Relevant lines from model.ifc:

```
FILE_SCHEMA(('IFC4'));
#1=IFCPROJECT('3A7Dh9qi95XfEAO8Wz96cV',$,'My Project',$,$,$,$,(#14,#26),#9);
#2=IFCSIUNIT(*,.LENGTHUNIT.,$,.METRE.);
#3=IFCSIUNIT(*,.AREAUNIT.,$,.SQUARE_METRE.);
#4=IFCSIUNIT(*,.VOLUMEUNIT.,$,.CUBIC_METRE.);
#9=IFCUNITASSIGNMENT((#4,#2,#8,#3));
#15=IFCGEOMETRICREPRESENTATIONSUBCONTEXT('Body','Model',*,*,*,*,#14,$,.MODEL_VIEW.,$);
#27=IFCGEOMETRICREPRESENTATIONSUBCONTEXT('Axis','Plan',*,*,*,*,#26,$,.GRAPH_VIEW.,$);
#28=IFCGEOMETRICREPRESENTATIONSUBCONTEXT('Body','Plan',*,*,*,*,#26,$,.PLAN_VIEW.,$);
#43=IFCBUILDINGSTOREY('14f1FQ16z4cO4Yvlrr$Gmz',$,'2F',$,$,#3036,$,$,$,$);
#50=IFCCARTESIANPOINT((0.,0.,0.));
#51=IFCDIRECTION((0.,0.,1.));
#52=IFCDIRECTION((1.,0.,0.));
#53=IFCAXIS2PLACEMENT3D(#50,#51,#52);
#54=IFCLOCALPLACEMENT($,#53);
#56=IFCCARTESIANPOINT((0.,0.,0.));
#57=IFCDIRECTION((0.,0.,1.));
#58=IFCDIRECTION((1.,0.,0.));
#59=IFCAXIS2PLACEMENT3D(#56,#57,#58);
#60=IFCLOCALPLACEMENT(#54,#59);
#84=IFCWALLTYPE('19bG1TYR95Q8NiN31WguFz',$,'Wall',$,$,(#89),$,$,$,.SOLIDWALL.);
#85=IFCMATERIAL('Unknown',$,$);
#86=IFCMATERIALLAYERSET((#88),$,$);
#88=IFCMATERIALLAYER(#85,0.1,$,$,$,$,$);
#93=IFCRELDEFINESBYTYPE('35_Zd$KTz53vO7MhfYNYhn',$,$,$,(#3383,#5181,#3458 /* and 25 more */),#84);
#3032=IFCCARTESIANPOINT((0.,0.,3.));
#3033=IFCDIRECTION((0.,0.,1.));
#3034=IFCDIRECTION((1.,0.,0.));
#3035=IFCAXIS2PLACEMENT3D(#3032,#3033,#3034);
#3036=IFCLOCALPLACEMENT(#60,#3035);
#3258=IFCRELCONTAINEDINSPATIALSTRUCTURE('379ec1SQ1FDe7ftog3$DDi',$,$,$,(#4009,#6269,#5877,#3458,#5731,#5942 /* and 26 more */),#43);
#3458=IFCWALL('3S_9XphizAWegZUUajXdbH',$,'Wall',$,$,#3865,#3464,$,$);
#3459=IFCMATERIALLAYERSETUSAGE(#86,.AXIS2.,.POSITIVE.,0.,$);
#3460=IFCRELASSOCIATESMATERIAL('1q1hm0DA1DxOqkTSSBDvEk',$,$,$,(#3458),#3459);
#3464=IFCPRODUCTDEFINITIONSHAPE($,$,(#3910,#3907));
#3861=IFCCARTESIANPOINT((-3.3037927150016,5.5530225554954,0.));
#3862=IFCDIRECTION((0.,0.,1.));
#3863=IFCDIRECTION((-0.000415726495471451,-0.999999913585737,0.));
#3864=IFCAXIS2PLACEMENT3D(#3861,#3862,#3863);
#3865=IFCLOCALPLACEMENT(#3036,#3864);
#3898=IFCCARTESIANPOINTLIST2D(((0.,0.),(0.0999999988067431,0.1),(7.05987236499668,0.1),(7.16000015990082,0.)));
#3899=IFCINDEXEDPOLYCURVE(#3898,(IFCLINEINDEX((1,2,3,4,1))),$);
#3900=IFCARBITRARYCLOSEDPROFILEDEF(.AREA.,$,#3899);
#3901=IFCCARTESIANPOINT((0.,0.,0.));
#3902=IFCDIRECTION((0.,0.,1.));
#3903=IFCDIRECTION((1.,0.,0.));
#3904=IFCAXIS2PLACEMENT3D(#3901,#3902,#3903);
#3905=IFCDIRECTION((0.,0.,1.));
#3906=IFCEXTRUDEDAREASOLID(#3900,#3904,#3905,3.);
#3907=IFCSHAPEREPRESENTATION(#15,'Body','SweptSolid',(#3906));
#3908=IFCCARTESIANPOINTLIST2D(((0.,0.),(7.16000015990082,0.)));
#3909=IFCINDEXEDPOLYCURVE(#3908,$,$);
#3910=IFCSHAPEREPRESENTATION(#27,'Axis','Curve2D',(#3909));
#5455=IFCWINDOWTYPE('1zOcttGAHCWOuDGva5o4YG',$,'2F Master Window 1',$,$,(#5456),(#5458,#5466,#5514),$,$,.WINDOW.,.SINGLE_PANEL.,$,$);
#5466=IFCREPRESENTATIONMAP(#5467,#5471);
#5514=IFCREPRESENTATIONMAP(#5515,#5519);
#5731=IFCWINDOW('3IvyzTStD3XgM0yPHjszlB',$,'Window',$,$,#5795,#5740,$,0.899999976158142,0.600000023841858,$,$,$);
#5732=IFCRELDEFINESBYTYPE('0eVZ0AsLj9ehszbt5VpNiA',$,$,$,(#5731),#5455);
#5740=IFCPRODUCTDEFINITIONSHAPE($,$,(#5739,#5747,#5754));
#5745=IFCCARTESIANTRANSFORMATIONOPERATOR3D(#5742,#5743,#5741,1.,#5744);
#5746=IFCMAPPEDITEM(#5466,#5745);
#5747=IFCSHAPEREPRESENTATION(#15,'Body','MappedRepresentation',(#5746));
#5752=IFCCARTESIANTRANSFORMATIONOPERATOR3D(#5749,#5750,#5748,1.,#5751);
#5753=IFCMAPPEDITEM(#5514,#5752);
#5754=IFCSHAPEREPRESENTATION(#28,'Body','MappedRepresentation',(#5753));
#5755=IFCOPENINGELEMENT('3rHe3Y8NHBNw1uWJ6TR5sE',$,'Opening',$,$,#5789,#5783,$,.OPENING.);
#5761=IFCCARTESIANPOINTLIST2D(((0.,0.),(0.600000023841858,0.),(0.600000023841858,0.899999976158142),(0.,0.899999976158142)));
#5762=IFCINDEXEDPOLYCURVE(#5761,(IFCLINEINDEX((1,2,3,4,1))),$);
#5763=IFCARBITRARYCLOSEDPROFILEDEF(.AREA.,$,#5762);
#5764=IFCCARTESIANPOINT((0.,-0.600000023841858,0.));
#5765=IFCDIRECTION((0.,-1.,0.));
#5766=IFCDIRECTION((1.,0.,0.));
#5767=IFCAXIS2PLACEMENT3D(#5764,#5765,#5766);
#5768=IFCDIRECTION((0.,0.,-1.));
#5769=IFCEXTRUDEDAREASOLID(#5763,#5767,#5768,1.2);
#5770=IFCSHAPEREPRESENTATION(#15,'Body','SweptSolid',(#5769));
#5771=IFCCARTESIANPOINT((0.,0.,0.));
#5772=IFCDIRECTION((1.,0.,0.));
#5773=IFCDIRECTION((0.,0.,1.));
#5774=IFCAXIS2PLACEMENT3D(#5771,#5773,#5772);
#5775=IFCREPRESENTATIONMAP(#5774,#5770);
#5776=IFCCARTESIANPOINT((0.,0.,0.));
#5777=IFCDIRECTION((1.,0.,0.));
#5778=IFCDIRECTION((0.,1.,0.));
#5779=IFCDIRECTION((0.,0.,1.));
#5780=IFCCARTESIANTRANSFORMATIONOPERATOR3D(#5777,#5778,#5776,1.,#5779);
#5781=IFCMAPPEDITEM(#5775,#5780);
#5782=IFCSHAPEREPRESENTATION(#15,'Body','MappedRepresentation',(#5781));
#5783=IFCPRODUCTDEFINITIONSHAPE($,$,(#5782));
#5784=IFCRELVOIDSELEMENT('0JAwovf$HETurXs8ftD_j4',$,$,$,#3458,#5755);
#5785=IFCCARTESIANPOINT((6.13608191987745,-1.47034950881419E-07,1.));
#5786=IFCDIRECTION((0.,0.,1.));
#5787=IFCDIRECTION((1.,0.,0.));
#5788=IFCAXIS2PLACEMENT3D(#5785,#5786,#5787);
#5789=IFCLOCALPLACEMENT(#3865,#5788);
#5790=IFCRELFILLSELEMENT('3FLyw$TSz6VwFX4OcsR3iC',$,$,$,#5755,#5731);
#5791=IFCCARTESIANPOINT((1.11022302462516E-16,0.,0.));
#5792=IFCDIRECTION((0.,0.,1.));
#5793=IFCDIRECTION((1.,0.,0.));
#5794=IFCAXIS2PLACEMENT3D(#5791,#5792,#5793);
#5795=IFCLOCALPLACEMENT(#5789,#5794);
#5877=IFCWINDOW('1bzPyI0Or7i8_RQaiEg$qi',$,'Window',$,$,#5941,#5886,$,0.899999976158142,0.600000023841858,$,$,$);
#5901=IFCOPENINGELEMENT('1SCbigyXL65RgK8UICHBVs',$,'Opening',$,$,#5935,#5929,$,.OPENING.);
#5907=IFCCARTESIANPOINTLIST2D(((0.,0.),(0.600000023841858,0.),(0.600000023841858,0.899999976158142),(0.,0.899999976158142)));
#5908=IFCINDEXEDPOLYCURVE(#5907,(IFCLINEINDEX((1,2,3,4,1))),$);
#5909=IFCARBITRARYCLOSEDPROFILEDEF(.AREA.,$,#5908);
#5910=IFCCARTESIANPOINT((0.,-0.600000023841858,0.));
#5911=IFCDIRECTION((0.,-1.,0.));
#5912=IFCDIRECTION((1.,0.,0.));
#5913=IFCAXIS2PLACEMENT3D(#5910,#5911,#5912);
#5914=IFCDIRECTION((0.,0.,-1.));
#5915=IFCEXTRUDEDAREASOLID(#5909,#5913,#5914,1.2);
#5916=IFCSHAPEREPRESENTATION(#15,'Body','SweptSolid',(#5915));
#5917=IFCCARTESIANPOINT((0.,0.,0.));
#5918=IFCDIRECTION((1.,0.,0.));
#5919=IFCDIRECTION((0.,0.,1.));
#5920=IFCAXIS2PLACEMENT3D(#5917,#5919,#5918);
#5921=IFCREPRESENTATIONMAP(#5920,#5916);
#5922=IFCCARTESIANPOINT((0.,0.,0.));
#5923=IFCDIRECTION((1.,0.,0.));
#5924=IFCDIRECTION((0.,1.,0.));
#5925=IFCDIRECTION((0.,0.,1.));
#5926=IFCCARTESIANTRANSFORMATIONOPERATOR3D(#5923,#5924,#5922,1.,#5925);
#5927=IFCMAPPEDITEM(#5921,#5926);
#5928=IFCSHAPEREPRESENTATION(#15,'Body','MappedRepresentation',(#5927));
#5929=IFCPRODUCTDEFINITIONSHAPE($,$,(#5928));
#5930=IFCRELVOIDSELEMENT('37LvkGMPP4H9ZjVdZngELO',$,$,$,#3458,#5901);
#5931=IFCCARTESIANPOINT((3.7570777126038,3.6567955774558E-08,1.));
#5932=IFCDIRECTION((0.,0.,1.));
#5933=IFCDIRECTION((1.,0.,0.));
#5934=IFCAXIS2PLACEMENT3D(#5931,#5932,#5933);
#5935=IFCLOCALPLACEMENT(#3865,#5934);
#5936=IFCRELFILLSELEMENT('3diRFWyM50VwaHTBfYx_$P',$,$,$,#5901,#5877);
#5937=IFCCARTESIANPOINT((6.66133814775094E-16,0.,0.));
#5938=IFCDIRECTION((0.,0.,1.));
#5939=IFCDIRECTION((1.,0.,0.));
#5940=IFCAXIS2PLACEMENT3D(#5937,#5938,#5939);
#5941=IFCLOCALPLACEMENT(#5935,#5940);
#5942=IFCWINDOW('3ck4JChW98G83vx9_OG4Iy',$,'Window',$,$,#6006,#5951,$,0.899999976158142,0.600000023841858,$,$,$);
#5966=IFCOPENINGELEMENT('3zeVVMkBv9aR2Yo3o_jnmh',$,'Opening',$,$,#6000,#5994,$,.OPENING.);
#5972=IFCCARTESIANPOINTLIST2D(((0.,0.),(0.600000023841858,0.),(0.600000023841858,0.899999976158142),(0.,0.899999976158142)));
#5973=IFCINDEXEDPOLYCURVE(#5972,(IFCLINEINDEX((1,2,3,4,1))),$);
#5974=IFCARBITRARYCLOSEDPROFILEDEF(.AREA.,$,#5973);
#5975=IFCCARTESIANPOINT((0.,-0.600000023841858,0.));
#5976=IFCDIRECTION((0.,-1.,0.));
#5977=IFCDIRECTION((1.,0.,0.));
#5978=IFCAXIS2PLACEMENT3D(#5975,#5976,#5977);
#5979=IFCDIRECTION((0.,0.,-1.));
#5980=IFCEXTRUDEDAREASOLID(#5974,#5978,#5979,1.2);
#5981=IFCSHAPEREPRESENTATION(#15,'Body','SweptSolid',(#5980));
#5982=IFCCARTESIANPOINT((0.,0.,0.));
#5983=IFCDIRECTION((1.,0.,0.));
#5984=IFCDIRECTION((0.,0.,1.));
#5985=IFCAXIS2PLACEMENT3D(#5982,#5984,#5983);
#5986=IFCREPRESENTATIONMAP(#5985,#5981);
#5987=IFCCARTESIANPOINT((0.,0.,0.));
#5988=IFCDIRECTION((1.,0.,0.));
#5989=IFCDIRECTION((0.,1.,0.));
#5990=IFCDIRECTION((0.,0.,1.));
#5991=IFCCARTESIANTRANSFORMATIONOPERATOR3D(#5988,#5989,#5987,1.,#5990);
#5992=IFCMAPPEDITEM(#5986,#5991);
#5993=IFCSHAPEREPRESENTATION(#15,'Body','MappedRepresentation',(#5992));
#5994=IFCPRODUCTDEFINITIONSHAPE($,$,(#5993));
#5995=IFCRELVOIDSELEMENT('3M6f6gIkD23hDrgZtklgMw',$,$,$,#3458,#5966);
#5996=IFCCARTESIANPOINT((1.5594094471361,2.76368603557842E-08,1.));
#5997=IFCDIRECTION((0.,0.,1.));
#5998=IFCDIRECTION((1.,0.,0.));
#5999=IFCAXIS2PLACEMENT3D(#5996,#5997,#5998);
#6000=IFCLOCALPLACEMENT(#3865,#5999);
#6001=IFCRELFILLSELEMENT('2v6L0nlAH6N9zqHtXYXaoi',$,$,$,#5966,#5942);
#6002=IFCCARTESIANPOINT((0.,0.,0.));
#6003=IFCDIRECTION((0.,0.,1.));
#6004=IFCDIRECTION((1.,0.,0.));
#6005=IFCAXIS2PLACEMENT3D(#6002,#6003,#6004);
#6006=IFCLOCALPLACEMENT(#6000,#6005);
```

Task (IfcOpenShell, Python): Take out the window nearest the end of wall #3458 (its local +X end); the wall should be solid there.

```python
import ifcopenshell
import ifcopenshell.api.feature
import ifcopenshell.api.root
import ifcopenshell.geom
import ifcopenshell.util.shape

model = ifcopenshell.open("model.ifc")
settings = ifcopenshell.geom.settings()


def volume(element):
    """Net volume in cubic metres, openings subtracted."""
    shape = ifcopenshell.geom.create_shape(settings, element)
    return ifcopenshell.util.shape.get_volume(shape.geometry)


window = model.by_guid("3IvyzTStD3XgM0yPHjszlB")
opening = window.FillsVoids[0].RelatingOpeningElement
wall = opening.VoidsElements[0].RelatingBuildingElement
before = volume(wall)

ifcopenshell.api.root.remove_product(model, product=window)
ifcopenshell.api.feature.remove_feature(model, feature=opening)

after = volume(wall)

print(f"wall volume {before:.3f} -> {after:.3f} m3")

model.write("model_v2.ifc")
```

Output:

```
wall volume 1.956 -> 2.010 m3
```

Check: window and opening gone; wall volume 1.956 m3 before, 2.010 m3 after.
